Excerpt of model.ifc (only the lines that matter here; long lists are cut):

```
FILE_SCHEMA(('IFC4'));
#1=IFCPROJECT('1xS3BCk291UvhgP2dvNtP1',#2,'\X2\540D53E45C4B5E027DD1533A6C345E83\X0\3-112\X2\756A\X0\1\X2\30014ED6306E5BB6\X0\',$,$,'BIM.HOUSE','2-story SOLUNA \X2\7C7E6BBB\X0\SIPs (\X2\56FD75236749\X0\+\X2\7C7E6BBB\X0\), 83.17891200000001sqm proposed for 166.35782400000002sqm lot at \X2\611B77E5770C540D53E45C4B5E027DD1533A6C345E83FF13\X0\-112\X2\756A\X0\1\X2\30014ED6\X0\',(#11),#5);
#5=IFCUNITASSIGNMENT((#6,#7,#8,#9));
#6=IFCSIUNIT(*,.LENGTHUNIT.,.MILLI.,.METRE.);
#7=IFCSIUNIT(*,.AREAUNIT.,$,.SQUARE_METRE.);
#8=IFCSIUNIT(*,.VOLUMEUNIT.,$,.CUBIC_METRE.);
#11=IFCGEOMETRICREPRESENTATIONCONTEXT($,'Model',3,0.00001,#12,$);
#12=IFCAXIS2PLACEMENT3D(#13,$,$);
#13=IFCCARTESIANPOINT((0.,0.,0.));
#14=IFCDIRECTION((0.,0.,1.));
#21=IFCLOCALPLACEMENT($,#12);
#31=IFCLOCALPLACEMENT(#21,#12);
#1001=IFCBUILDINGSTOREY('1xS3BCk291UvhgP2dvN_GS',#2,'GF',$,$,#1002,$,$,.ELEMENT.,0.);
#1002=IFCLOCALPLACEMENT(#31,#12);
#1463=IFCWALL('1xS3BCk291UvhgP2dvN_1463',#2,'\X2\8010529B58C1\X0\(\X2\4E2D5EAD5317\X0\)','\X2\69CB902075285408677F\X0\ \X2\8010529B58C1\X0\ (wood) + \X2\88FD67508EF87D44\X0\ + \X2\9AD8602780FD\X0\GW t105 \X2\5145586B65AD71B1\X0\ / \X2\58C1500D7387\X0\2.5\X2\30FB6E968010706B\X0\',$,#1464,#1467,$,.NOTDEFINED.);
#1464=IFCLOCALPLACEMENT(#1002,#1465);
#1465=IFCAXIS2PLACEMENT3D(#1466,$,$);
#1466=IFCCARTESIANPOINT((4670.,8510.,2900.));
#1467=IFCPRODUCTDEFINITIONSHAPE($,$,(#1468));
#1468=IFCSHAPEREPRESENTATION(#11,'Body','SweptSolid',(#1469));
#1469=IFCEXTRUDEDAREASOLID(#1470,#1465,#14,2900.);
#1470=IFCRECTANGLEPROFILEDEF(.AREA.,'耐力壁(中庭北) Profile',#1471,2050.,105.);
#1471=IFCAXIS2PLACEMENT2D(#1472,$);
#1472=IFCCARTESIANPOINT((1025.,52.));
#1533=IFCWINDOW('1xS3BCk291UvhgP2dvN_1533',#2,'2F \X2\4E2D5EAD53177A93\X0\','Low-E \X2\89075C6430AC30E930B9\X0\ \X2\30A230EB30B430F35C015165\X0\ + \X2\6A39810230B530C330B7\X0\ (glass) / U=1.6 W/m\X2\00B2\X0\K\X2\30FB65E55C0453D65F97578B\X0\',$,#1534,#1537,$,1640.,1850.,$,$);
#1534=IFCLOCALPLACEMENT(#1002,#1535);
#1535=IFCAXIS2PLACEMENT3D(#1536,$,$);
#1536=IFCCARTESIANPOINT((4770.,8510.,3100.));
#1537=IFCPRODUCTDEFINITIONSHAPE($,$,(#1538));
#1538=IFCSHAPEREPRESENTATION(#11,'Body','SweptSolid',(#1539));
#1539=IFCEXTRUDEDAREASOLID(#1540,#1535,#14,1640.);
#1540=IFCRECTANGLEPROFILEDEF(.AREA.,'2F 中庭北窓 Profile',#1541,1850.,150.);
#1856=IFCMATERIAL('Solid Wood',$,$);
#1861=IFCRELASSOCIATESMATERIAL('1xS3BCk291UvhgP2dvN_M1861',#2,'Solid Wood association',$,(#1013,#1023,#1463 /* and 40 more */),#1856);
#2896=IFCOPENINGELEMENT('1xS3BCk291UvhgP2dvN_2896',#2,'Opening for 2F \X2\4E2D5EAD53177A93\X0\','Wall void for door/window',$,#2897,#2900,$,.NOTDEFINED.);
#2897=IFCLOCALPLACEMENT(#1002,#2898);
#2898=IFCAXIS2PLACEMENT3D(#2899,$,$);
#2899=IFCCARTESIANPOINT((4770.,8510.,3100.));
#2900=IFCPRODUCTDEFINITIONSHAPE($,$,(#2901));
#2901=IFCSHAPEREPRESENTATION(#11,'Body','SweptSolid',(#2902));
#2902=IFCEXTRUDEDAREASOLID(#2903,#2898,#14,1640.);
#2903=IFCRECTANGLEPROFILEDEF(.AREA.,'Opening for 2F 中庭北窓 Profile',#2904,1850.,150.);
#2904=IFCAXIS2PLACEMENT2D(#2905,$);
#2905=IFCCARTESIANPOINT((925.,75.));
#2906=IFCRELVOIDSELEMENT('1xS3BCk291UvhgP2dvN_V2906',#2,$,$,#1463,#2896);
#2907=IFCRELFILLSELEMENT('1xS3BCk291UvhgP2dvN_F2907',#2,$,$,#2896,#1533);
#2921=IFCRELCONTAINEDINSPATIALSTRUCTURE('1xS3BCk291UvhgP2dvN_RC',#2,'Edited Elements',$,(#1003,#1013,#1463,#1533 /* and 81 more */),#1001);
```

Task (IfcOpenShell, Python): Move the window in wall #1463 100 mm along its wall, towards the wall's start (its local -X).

```python
import ifcopenshell
import ifcopenshell.api.geometry
import ifcopenshell.util.placement

model = ifcopenshell.open("model.ifc")

window = model.by_guid("1xS3BCk291UvhgP2dvN_1533")
opening = window.FillsVoids[0].RelatingOpeningElement
wall = opening.VoidsElements[0].RelatingBuildingElement

wall_matrix = ifcopenshell.util.placement.get_local_placement(wall.ObjectPlacement)
shift = wall_matrix[:3, 0] * -100.0
before = ifcopenshell.util.placement.get_local_placement(window.ObjectPlacement)[:3, 3].copy()

# The window is not placed relative to its opening, so move both.
for product in (opening, window):
    matrix = ifcopenshell.util.placement.get_local_placement(product.ObjectPlacement)
    matrix[:3, 3] += shift
    ifcopenshell.api.geometry.edit_object_placement(model, product=product, matrix=matrix, is_si=False)

after = ifcopenshell.util.placement.get_local_placement(window.ObjectPlacement)[:3, 3]
print("window moved by", (after - before).round(3) + 0.0)

model.write("model-out.ifc")
```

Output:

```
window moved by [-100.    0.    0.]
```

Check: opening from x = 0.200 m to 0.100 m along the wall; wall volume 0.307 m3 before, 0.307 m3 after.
